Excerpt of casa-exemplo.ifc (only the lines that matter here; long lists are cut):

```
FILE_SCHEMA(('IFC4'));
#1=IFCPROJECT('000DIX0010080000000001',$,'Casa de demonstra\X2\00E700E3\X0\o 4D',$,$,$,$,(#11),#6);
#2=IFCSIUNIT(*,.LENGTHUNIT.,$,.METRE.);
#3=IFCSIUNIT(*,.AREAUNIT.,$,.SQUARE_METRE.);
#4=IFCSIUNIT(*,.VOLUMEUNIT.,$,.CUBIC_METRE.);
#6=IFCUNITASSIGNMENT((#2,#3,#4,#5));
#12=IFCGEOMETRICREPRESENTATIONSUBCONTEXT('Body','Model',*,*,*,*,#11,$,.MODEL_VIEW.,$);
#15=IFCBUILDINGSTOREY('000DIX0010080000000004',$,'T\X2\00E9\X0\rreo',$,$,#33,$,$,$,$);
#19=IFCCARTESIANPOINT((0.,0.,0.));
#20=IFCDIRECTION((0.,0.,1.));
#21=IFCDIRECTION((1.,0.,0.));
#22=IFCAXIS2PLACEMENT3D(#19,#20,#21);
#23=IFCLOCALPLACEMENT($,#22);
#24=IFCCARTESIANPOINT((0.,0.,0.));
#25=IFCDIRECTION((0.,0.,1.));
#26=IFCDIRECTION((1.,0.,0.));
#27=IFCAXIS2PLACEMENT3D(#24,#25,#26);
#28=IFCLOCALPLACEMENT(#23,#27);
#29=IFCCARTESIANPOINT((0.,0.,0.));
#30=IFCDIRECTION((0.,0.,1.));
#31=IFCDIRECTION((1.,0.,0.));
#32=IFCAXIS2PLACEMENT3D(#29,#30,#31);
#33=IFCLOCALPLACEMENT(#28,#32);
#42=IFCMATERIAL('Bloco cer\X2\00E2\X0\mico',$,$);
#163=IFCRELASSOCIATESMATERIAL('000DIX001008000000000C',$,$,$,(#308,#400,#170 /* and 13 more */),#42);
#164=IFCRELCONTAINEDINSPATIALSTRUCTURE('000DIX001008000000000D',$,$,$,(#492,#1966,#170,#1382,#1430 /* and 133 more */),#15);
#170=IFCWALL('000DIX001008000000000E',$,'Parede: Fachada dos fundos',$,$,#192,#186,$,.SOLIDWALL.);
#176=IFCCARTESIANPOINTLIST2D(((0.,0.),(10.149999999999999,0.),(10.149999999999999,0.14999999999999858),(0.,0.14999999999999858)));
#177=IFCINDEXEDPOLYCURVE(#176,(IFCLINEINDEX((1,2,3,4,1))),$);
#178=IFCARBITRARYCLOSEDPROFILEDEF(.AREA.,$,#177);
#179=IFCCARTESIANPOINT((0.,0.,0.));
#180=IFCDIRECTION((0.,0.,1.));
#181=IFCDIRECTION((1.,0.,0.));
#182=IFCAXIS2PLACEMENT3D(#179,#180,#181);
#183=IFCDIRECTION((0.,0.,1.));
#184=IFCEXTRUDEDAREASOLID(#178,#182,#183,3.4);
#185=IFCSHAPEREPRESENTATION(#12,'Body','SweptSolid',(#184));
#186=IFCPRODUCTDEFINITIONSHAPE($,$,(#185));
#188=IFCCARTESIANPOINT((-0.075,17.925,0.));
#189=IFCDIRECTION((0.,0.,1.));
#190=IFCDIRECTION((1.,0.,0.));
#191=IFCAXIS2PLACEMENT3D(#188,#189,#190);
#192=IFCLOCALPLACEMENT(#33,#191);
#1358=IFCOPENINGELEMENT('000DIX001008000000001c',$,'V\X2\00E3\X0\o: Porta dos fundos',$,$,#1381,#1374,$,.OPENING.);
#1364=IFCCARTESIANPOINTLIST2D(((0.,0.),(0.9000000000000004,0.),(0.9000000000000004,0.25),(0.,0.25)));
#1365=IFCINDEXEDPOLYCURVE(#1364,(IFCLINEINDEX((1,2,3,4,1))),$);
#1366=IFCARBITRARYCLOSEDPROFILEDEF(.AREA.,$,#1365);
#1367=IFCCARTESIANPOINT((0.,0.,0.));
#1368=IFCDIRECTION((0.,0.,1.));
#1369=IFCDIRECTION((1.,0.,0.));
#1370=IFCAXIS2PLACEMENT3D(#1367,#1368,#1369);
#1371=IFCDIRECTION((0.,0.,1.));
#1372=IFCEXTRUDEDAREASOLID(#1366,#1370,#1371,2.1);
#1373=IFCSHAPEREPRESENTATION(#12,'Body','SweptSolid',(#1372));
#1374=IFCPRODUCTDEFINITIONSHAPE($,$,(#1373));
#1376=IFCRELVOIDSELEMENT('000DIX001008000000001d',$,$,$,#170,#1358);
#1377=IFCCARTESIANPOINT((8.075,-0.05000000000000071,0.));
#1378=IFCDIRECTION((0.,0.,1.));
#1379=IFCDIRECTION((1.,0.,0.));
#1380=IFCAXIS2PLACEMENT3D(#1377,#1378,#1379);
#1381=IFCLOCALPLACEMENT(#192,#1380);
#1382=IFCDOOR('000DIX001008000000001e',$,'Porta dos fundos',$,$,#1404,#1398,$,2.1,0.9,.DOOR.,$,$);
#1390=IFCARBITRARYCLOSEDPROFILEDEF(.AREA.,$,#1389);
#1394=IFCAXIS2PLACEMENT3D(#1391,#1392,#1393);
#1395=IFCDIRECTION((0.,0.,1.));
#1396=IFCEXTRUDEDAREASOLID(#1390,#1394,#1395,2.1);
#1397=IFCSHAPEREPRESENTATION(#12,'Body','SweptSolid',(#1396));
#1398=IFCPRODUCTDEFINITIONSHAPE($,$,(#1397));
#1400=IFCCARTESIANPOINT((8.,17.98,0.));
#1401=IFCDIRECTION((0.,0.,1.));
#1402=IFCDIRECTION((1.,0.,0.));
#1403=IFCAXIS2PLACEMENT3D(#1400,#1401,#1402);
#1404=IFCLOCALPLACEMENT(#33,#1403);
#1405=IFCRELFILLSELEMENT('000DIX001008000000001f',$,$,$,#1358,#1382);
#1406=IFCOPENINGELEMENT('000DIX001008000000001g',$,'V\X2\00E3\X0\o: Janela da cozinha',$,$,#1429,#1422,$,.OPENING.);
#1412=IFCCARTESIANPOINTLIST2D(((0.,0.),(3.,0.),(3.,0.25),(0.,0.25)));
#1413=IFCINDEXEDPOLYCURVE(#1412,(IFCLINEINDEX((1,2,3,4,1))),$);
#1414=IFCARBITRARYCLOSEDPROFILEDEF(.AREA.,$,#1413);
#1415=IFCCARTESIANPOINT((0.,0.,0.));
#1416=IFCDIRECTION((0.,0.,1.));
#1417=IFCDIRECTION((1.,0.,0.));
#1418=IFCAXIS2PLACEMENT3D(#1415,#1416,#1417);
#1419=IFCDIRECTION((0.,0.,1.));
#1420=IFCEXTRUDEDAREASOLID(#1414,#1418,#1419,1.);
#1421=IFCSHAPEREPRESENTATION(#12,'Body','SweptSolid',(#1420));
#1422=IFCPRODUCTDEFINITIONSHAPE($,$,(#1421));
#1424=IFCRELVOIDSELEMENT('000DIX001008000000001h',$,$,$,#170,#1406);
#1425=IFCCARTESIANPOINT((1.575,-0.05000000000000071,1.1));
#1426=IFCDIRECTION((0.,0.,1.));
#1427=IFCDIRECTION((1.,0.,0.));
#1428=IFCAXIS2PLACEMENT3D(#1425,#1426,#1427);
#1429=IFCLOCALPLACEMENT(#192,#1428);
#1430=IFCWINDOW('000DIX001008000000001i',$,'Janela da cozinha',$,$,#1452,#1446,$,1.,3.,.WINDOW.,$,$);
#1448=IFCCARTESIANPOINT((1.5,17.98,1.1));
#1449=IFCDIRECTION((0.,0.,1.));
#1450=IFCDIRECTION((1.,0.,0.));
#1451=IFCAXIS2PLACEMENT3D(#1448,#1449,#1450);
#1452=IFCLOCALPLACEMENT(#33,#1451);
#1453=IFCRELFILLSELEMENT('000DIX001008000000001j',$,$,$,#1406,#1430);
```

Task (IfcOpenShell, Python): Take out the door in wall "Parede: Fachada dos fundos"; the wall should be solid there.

```python
import ifcopenshell
import ifcopenshell.api.feature
import ifcopenshell.api.root
import ifcopenshell.geom
import ifcopenshell.util.shape

model = ifcopenshell.open("casa-exemplo.ifc")
settings = ifcopenshell.geom.settings()


def volume(element):
    """Net volume in cubic metres, openings subtracted."""
    shape = ifcopenshell.geom.create_shape(settings, element)
    return ifcopenshell.util.shape.get_volume(shape.geometry)


door = model.by_guid("000DIX001008000000001e")
opening = door.FillsVoids[0].RelatingOpeningElement
wall = opening.VoidsElements[0].RelatingBuildingElement
before = volume(wall)

ifcopenshell.api.root.remove_product(model, product=door)
ifcopenshell.api.feature.remove_feature(model, feature=opening)

after = volume(wall)

print(f"wall volume {before:.3f} -> {after:.3f} m3")

model.write("casa-exemplo_v2.ifc")
```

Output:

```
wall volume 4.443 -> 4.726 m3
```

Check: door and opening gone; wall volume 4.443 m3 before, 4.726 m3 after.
